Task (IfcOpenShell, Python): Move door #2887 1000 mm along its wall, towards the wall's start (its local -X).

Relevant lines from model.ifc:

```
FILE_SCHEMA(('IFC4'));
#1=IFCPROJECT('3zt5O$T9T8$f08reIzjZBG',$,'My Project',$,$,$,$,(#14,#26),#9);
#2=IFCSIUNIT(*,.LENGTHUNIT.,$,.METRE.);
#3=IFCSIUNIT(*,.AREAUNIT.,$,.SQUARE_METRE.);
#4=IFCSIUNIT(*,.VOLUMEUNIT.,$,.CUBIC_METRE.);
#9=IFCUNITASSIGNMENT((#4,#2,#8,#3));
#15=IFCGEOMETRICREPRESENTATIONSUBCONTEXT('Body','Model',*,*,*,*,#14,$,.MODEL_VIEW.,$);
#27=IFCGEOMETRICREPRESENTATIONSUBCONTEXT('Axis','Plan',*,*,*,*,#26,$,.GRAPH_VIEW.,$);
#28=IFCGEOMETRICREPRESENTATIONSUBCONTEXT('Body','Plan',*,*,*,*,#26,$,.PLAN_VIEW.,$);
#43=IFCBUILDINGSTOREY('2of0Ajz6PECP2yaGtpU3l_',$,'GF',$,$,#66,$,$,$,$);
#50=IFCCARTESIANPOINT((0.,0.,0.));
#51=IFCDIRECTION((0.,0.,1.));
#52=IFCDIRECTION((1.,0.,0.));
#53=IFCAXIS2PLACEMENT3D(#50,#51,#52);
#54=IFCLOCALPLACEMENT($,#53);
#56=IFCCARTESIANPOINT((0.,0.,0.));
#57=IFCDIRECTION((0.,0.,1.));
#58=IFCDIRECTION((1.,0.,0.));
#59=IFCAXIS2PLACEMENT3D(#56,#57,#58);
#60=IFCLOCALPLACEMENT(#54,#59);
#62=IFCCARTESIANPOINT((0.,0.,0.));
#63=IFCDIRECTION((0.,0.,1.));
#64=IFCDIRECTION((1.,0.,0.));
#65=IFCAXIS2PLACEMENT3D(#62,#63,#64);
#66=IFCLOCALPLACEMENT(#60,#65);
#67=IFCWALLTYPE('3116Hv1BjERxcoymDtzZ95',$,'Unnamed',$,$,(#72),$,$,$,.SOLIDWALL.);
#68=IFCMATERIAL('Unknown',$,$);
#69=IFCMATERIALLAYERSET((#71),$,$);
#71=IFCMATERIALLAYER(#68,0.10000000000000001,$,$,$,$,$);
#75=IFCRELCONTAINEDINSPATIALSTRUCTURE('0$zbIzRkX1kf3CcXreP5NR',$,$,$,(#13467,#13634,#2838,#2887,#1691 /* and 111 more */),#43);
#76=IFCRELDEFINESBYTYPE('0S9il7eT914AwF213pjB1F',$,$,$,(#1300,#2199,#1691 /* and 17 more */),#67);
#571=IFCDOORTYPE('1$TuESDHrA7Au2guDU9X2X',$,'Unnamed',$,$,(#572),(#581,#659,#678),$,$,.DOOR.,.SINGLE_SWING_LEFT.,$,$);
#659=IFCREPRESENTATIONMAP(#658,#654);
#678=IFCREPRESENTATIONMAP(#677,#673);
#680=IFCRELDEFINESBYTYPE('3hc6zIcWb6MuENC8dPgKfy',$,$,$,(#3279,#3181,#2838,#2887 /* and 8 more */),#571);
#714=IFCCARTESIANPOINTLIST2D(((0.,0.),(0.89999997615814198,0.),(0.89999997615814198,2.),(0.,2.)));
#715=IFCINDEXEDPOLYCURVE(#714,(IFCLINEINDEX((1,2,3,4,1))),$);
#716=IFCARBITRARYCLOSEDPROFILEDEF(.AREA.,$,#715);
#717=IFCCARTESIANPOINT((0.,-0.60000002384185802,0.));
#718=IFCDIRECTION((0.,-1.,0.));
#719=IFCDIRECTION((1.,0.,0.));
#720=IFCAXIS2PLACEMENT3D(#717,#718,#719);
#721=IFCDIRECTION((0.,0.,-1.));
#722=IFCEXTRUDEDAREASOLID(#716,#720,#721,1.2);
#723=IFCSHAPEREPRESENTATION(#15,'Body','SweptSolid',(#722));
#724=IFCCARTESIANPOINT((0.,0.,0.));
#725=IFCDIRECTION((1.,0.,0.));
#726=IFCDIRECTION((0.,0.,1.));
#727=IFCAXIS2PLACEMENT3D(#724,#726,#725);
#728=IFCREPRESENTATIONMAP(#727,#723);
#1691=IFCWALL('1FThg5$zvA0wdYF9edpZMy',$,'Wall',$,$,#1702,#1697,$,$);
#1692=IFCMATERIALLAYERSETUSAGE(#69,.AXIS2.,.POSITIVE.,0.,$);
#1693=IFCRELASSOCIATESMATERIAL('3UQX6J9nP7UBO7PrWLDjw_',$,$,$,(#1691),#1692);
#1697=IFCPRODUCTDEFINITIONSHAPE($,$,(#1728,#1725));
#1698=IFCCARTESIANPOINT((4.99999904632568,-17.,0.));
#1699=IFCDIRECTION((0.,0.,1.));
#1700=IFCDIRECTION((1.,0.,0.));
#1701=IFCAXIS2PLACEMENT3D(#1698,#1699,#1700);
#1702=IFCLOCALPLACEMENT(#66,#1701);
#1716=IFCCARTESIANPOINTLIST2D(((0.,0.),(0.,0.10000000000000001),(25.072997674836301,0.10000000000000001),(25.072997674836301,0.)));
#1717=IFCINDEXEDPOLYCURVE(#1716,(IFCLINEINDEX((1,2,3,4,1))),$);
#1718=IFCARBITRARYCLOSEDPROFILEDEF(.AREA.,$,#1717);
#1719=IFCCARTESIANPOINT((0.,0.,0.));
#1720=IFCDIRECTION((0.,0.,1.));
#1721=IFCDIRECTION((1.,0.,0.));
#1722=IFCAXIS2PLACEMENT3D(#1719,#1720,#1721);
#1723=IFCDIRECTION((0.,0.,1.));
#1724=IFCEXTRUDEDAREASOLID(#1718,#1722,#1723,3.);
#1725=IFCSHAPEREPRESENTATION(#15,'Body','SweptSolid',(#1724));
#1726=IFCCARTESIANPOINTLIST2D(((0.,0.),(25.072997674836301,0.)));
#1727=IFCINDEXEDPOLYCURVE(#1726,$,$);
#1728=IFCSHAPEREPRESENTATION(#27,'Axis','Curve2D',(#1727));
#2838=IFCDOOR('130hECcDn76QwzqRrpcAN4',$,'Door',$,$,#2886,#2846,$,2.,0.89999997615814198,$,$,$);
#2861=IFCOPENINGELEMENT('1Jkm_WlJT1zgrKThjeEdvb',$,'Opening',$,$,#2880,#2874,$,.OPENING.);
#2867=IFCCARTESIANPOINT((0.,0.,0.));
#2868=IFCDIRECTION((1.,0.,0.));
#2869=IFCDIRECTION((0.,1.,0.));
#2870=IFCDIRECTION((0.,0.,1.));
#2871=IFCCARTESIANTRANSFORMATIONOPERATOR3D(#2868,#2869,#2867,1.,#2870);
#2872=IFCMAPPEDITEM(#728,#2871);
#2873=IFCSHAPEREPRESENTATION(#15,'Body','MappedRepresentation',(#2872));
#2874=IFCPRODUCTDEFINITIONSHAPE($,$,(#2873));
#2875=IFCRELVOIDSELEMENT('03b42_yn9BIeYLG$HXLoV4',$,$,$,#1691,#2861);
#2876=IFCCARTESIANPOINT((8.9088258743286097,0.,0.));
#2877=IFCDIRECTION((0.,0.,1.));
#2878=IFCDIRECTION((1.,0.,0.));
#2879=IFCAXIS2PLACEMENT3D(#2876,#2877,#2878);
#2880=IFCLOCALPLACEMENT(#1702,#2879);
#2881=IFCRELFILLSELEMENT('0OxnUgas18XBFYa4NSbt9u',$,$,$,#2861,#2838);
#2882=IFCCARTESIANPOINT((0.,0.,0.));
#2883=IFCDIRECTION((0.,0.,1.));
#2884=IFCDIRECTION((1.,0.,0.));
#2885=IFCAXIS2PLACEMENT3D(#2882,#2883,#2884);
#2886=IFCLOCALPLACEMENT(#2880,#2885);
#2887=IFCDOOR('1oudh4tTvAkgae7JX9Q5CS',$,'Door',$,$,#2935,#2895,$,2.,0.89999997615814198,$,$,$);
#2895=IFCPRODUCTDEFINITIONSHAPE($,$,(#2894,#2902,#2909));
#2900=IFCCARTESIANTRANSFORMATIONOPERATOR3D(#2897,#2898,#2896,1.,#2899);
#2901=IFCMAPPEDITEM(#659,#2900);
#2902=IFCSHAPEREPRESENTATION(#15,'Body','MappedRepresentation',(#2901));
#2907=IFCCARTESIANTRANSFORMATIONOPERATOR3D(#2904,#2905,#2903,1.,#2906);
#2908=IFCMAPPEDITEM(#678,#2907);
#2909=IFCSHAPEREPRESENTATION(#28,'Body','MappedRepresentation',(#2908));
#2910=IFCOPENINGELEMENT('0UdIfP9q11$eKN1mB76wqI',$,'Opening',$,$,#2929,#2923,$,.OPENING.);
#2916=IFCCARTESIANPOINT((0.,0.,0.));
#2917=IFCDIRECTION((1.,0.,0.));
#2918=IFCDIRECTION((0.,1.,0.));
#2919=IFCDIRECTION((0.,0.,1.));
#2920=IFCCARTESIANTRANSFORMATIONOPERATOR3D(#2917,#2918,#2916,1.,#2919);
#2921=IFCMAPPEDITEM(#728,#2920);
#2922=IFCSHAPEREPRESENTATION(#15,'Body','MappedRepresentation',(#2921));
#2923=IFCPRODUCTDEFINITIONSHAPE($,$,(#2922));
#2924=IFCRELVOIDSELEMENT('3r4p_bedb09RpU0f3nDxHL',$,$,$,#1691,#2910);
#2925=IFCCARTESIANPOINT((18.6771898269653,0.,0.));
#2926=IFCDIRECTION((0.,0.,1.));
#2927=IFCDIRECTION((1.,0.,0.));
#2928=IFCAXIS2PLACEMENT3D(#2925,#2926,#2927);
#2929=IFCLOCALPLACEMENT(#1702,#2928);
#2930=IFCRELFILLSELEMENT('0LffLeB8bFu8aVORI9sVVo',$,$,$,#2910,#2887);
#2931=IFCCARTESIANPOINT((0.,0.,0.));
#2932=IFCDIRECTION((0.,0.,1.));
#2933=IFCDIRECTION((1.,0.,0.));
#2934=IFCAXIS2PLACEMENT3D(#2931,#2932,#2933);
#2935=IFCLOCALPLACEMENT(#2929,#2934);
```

```python
import ifcopenshell
import ifcopenshell.api.geometry
import ifcopenshell.util.placement

model = ifcopenshell.open("model.ifc")

door = model.by_guid("1oudh4tTvAkgae7JX9Q5CS")
opening = door.FillsVoids[0].RelatingOpeningElement
wall = opening.VoidsElements[0].RelatingBuildingElement

wall_matrix = ifcopenshell.util.placement.get_local_placement(wall.ObjectPlacement)
shift = wall_matrix[:3, 0] * -1.0
before = ifcopenshell.util.placement.get_local_placement(door.ObjectPlacement)[:3, 3].copy()

# The door is placed relative to its opening, so it follows when the opening moves.
matrix = ifcopenshell.util.placement.get_local_placement(opening.ObjectPlacement)
matrix[:3, 3] += shift
ifcopenshell.api.geometry.edit_object_placement(
    model, product=opening, matrix=matrix, is_si=False, should_transform_children=True
)

after = ifcopenshell.util.placement.get_local_placement(door.ObjectPlacement)[:3, 3]
print("door moved by", (after - before).round(3) + 0.0)

model.write("model_updated.ifc")
```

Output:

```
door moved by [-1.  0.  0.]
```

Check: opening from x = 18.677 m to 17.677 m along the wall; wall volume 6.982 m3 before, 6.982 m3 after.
